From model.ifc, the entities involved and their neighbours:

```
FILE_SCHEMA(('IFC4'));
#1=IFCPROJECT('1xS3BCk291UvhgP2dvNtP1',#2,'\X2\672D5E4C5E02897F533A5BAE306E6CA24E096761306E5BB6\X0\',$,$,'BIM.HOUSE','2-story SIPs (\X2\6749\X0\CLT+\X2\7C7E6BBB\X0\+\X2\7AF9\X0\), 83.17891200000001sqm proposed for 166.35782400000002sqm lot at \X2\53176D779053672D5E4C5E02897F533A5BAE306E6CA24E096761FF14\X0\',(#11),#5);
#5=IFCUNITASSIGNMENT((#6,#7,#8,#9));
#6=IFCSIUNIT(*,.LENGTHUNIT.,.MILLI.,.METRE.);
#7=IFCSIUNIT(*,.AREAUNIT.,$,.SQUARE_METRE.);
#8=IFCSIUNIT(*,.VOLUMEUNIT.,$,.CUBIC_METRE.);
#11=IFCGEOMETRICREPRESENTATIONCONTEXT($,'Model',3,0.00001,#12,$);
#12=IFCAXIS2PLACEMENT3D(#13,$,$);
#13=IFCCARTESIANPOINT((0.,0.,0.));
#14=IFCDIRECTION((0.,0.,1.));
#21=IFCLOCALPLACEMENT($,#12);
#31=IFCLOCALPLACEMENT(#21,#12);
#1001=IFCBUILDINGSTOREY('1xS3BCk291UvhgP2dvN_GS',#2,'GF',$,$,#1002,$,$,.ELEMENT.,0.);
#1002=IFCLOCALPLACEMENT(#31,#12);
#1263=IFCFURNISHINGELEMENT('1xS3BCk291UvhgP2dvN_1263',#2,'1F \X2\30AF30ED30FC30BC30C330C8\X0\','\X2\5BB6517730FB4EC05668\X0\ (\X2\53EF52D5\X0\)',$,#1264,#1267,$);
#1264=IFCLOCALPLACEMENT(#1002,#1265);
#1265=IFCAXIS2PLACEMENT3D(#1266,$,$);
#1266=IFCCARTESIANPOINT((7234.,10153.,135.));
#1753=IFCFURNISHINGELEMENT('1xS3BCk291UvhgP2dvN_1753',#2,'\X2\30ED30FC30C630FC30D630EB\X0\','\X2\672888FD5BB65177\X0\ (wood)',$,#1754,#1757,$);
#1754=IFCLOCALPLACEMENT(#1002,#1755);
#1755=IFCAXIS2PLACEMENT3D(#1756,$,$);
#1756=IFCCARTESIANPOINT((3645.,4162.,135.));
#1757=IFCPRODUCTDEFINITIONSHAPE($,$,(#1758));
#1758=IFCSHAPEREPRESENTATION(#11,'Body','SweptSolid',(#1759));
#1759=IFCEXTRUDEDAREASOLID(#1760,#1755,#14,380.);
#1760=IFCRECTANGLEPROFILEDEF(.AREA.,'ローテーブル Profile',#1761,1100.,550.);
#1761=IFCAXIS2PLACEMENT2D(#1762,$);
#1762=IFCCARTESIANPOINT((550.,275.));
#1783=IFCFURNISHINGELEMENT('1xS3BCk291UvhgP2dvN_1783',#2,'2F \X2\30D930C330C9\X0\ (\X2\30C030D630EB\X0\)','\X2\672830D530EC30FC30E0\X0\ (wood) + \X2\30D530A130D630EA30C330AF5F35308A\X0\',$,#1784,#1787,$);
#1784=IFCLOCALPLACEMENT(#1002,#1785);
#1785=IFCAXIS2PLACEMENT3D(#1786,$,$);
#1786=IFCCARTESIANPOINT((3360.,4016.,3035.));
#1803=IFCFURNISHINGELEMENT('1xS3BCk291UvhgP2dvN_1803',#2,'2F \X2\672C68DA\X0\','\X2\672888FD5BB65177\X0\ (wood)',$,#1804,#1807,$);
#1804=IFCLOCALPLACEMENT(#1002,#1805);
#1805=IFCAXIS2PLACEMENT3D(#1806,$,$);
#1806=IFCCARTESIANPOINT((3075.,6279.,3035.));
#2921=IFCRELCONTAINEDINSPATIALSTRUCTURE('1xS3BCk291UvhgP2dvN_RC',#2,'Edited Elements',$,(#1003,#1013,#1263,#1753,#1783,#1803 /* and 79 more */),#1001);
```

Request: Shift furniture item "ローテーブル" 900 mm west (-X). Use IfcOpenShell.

```python
import ifcopenshell
import ifcopenshell.api.geometry
import ifcopenshell.util.placement

model = ifcopenshell.open("model.ifc")

item = model.by_id(1753)
matrix = ifcopenshell.util.placement.get_local_placement(item.ObjectPlacement)
matrix[0, 3] -= 900.0
ifcopenshell.api.geometry.edit_object_placement(model, product=item, matrix=matrix, is_si=False)

print(ifcopenshell.util.placement.get_local_placement(item.ObjectPlacement).round(3) + 0.0)

model.write("model_updated.ifc")
```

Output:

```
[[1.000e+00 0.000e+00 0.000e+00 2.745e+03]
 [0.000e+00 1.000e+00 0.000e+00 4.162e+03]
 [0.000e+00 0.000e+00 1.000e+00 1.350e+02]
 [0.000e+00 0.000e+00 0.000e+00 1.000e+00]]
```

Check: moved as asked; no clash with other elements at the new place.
